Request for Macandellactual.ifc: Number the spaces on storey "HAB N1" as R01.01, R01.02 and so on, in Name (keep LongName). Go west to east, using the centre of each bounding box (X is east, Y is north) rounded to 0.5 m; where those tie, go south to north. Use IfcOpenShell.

First a look at what the model holds.

```python
import ifcopenshell
import ifcopenshell.util.element
import ifcopenshell.util.placement

model = ifcopenshell.open("Macandellactual.ifc")
print(model.schema)
storey = next(s for s in model.by_type("IfcBuildingStorey") if s.Name == "HAB N1")
spaces = [e for e in ifcopenshell.util.element.get_decomposition(storey) if e.is_a("IfcSpace")]
for e in sorted(spaces, key=lambda e: e.id()):
    origin = ifcopenshell.util.placement.get_local_placement(e.ObjectPlacement)[:3, 3]
    print(e.id(), e.Name, e.LongName, origin.round(2) + 0.0, sep=" | ")
```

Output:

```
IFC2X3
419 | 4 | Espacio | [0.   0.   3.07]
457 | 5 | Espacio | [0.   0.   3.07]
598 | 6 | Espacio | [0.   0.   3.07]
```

```python
import ifcopenshell
import ifcopenshell.geom
import ifcopenshell.util.element
import ifcopenshell.util.shape

model = ifcopenshell.open("Macandellactual.ifc")
settings = ifcopenshell.geom.settings()
settings.set("use-world-coords", True)


def centre(element):
    shape = ifcopenshell.geom.create_shape(settings, element)
    return ifcopenshell.util.shape.get_bbox_centroid(shape.geometry)


storey = next(s for s in model.by_type("IfcBuildingStorey") if s.Name == "HAB N1")
spaces = [e for e in ifcopenshell.util.element.get_decomposition(storey) if e.is_a("IfcSpace")]

# Insertion points can sit at a corner or the storey origin, so sort by the geometry (in metres).
centres = {e: centre(e) for e in spaces}
spaces.sort(key=lambda e: (round(centres[e][0] / 0.5), centres[e][1]))

for i, e in enumerate(spaces, start=1):
    number = f"R01.{i:02d}"
    e.Name = number
    print(e.id(), number)

model.write("Macandellactual_updated.ifc")
```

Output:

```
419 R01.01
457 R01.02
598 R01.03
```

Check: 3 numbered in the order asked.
